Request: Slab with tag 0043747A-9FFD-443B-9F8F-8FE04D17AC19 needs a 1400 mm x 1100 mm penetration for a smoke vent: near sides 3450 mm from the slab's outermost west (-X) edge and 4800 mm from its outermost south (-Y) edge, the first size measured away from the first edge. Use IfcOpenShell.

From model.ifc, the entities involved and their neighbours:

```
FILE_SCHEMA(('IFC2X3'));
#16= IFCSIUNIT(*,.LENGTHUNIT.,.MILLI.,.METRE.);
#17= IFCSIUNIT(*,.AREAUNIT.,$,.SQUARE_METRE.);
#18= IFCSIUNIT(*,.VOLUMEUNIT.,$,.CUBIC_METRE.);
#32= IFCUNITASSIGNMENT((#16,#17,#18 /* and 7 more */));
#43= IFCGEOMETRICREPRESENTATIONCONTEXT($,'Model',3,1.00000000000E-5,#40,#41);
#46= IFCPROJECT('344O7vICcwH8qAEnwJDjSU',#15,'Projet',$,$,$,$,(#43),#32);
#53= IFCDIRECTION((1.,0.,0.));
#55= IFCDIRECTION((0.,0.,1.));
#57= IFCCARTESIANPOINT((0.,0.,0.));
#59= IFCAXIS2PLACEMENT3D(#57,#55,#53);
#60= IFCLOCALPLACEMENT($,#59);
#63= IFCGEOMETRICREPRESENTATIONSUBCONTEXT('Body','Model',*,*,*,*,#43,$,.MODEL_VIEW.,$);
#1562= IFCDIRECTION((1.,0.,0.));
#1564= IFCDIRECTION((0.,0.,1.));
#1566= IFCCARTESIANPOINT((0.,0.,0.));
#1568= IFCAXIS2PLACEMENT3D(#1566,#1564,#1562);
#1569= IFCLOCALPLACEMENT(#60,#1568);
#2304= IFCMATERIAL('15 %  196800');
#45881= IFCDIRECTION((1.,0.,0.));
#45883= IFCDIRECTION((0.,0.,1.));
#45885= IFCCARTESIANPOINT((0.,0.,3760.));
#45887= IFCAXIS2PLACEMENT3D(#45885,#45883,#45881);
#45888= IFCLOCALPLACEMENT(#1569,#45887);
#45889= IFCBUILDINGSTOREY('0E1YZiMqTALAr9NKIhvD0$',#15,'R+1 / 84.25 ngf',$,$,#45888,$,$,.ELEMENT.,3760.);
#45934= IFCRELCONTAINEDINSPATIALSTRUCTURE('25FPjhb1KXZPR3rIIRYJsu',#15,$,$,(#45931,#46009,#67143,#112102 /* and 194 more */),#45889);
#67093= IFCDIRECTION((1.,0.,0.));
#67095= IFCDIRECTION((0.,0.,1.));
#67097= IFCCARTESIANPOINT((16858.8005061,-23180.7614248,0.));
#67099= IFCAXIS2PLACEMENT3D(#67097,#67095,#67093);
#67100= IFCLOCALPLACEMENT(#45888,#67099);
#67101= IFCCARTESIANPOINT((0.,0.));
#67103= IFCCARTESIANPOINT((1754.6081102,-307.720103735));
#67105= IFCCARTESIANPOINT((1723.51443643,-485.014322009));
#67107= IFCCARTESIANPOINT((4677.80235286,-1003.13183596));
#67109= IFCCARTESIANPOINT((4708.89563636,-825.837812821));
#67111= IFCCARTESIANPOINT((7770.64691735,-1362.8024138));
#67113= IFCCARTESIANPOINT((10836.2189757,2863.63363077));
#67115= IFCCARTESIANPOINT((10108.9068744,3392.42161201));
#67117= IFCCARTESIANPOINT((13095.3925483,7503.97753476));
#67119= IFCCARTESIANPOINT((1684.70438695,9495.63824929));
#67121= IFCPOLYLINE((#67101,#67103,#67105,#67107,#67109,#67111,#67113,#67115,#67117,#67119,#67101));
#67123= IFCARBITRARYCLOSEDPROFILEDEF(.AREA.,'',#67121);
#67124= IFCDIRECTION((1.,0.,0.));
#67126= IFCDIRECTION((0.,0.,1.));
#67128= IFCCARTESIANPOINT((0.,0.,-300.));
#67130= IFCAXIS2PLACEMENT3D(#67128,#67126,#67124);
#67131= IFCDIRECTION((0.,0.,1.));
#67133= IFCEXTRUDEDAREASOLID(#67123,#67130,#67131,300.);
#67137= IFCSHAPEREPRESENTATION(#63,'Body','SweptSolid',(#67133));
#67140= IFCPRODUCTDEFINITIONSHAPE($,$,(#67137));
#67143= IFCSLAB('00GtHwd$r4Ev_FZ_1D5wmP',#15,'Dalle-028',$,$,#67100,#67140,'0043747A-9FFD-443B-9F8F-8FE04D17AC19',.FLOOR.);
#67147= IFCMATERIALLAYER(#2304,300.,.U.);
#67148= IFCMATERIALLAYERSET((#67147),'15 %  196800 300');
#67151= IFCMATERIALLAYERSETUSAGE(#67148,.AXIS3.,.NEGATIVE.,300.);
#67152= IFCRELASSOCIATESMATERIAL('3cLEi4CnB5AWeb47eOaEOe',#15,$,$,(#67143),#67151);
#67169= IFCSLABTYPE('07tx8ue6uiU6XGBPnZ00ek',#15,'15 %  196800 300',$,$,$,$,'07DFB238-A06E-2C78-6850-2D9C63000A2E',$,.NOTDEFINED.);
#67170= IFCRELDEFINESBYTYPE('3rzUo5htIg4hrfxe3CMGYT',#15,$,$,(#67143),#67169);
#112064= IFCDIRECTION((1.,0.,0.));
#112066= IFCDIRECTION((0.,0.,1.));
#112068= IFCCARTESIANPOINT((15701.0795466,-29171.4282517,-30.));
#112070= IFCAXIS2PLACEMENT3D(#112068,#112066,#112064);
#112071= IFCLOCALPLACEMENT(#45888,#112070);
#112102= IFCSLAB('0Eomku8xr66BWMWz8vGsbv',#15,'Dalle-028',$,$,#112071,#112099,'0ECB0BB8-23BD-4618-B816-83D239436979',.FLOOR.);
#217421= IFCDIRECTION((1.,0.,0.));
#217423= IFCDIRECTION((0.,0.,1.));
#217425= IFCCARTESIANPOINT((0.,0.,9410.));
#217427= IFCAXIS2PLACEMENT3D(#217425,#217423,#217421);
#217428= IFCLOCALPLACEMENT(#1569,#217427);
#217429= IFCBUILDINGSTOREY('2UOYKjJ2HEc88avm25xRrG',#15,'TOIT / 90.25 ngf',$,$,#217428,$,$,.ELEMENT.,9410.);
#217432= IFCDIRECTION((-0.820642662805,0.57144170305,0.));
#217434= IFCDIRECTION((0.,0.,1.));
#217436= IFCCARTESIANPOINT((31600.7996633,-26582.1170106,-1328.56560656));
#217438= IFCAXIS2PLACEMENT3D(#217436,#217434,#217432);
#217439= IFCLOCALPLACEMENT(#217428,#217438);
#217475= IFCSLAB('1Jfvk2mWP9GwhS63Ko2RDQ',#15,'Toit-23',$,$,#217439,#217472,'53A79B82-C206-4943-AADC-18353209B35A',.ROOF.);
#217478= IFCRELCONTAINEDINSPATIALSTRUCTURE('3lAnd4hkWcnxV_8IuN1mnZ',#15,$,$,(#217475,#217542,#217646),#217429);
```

```python
import numpy as np
import ifcopenshell
import ifcopenshell.api.feature
import ifcopenshell.api.geometry
import ifcopenshell.api.root
import ifcopenshell.geom
import ifcopenshell.util.placement
import ifcopenshell.util.representation
import ifcopenshell.util.shape
import ifcopenshell.util.unit

model = ifcopenshell.open("model.ifc")
unit_scale = ifcopenshell.util.unit.calculate_unit_scale(model)
settings = ifcopenshell.geom.settings()


def volume(element):
    """Net volume in cubic metres, openings subtracted."""
    shape = ifcopenshell.geom.create_shape(settings, element)
    return ifcopenshell.util.shape.get_volume(shape.geometry)


slab = model.by_id(67143)
before = volume(slab)

# Extent in the slab's own axes, in metres. The edges named are its -X and -Y sides.
slab_shape = ifcopenshell.geom.create_shape(settings, slab)
vertices = ifcopenshell.util.shape.get_vertices(slab_shape.geometry)
x_min, y_min, bottom = vertices.min(axis=0)
top = vertices[:, 2].max()

opening = ifcopenshell.api.root.create_entity(model, ifc_class="IfcOpeningElement", name="Smoke vent opening")
context = ifcopenshell.util.representation.get_context(model, "Model", "Body", "MODEL_VIEW")
width, depth = 1.4, 1.1
outline = [(0.0, 0.0), (width, 0.0), (width, depth), (0.0, depth), (0.0, 0.0)]
# Overshoot both faces by 50 mm so the cut is clean.
shape = ifcopenshell.api.geometry.add_slab_representation(
    model, context=context, depth=top - bottom + 0.1, polyline=outline
)
ifcopenshell.api.geometry.assign_representation(model, product=opening, representation=shape)

matrix = ifcopenshell.util.placement.get_local_placement(slab.ObjectPlacement)
matrix[:, 3] = matrix @ np.append(np.array([x_min + 3.45, y_min + 4.8, bottom - 0.05]) / unit_scale, 1.0)
ifcopenshell.api.geometry.edit_object_placement(model, product=opening, matrix=matrix, is_si=False)
ifcopenshell.api.feature.add_feature(model, feature=opening, element=slab)

after = volume(slab)

print(f"slab volume {before:.3f} -> {after:.3f} m3")

model.write("model_updated.ifc")
```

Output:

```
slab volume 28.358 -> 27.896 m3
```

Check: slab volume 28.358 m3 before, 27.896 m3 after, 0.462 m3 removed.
